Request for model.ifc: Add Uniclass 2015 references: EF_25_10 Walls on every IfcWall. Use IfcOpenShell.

First a look at what the model holds.

```python
import ifcopenshell

model = ifcopenshell.open("model.ifc")
print(model.schema)
print("classifications:", [c.Name for c in model.by_type("IfcClassification")])
for ifc_class in ("IfcDoor", "IfcRoof", "IfcStair", "IfcWall", "IfcWindow"):
    print(ifc_class, len(model.by_type(ifc_class)))
```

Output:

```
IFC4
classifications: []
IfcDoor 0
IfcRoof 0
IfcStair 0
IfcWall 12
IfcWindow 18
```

```python
import ifcopenshell
import ifcopenshell.api.classification

model = ifcopenshell.open("model.ifc")

system = ifcopenshell.api.classification.add_classification(model, classification="Uniclass 2015")

codes = {
    "IfcWall": ("EF_25_10", "Walls"),
}
for ifc_class, (code, name) in codes.items():
    products = model.by_type(ifc_class)
    ifcopenshell.api.classification.add_reference(
        model, products=products, classification=system, identification=code, name=name
    )
    print(code, len(products))

model.write("model_v2.ifc")
```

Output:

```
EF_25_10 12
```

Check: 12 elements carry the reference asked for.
